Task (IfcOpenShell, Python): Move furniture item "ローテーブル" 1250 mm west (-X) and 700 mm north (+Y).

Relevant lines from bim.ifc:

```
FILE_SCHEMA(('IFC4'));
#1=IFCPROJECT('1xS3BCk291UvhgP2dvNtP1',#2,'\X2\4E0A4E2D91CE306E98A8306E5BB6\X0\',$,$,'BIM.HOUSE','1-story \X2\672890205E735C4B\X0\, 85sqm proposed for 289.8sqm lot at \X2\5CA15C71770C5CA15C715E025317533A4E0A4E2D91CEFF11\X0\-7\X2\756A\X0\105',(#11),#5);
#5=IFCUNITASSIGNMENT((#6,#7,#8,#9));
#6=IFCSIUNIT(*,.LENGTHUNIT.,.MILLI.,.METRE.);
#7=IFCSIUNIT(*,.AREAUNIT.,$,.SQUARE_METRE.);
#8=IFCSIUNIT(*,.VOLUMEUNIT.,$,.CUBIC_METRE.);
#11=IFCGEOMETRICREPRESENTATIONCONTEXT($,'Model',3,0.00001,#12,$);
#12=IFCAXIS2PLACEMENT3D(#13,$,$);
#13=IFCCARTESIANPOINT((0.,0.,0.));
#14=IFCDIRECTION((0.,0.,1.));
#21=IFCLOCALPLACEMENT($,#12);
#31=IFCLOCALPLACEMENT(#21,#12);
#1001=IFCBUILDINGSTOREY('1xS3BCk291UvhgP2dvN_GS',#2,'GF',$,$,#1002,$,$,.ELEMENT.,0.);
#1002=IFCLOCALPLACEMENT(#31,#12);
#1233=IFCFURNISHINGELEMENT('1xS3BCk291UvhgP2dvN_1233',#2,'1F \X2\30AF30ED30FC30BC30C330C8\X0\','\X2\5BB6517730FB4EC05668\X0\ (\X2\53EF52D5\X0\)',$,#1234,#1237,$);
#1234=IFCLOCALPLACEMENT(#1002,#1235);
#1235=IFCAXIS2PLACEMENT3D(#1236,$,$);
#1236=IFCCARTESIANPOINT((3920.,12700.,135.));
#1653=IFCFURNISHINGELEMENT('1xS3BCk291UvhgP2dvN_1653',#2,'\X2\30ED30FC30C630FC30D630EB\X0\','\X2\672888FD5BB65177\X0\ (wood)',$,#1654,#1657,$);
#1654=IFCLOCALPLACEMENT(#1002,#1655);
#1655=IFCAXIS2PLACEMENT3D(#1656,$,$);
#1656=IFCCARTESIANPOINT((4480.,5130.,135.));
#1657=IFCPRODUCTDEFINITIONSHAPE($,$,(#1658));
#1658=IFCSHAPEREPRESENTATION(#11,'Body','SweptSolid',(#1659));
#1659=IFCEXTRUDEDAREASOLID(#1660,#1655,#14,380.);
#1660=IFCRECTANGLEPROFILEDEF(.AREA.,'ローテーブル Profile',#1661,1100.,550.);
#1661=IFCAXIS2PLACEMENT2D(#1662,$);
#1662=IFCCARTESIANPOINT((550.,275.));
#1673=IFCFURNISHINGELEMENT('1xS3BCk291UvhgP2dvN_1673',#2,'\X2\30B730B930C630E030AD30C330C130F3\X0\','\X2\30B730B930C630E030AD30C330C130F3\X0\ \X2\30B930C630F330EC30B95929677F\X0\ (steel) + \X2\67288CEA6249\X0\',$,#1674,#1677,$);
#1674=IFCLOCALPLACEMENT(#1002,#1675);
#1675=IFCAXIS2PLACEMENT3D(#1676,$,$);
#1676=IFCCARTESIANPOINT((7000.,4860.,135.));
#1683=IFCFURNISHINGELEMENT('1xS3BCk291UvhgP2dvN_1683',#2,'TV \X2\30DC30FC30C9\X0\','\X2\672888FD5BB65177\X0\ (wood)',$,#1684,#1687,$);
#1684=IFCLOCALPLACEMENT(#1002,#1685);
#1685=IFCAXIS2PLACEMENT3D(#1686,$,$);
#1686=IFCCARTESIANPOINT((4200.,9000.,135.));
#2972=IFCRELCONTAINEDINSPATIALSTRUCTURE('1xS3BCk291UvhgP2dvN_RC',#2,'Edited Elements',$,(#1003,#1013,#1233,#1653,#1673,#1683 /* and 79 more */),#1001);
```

```python
import ifcopenshell
import ifcopenshell.api.geometry
import ifcopenshell.util.placement
import ifcopenshell.util.unit

model = ifcopenshell.open("bim.ifc")
unit_scale = ifcopenshell.util.unit.calculate_unit_scale(model)

item = model.by_id(1653)
matrix = ifcopenshell.util.placement.get_local_placement(item.ObjectPlacement)
matrix[0, 3] -= 1.25 / unit_scale
matrix[1, 3] += 0.7 / unit_scale
ifcopenshell.api.geometry.edit_object_placement(model, product=item, matrix=matrix, is_si=False)

print(ifcopenshell.util.placement.get_local_placement(item.ObjectPlacement).round(3) + 0.0)

model.write("bim_updated.ifc")
```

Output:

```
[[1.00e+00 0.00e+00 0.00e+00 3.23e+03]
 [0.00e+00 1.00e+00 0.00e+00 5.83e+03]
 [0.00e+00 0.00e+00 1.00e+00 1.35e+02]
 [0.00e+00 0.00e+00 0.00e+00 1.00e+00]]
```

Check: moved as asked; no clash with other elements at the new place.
